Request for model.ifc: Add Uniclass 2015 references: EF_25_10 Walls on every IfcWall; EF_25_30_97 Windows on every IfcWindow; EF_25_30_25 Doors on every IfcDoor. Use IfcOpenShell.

First a look at what the model holds.

```python
import ifcopenshell

model = ifcopenshell.open("model.ifc")
print(model.schema)
print("classifications:", [c.Name for c in model.by_type("IfcClassification")])
for ifc_class in ("IfcDoor", "IfcRoof", "IfcStair", "IfcWall", "IfcWindow"):
    print(ifc_class, len(model.by_type(ifc_class)))
```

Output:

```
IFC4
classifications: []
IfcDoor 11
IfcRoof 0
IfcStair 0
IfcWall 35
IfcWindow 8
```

```python
import ifcopenshell
import ifcopenshell.api.classification

model = ifcopenshell.open("model.ifc")

system = ifcopenshell.api.classification.add_classification(model, classification="Uniclass 2015")

codes = {
    "IfcWall": ("EF_25_10", "Walls"),
    "IfcWindow": ("EF_25_30_97", "Windows"),
    "IfcDoor": ("EF_25_30_25", "Doors"),
}
for ifc_class, (code, name) in codes.items():
    products = model.by_type(ifc_class)
    ifcopenshell.api.classification.add_reference(
        model, products=products, classification=system, identification=code, name=name
    )
    print(code, len(products))

model.write("model_edited.ifc")
```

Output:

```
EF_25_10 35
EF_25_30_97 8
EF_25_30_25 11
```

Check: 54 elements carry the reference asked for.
